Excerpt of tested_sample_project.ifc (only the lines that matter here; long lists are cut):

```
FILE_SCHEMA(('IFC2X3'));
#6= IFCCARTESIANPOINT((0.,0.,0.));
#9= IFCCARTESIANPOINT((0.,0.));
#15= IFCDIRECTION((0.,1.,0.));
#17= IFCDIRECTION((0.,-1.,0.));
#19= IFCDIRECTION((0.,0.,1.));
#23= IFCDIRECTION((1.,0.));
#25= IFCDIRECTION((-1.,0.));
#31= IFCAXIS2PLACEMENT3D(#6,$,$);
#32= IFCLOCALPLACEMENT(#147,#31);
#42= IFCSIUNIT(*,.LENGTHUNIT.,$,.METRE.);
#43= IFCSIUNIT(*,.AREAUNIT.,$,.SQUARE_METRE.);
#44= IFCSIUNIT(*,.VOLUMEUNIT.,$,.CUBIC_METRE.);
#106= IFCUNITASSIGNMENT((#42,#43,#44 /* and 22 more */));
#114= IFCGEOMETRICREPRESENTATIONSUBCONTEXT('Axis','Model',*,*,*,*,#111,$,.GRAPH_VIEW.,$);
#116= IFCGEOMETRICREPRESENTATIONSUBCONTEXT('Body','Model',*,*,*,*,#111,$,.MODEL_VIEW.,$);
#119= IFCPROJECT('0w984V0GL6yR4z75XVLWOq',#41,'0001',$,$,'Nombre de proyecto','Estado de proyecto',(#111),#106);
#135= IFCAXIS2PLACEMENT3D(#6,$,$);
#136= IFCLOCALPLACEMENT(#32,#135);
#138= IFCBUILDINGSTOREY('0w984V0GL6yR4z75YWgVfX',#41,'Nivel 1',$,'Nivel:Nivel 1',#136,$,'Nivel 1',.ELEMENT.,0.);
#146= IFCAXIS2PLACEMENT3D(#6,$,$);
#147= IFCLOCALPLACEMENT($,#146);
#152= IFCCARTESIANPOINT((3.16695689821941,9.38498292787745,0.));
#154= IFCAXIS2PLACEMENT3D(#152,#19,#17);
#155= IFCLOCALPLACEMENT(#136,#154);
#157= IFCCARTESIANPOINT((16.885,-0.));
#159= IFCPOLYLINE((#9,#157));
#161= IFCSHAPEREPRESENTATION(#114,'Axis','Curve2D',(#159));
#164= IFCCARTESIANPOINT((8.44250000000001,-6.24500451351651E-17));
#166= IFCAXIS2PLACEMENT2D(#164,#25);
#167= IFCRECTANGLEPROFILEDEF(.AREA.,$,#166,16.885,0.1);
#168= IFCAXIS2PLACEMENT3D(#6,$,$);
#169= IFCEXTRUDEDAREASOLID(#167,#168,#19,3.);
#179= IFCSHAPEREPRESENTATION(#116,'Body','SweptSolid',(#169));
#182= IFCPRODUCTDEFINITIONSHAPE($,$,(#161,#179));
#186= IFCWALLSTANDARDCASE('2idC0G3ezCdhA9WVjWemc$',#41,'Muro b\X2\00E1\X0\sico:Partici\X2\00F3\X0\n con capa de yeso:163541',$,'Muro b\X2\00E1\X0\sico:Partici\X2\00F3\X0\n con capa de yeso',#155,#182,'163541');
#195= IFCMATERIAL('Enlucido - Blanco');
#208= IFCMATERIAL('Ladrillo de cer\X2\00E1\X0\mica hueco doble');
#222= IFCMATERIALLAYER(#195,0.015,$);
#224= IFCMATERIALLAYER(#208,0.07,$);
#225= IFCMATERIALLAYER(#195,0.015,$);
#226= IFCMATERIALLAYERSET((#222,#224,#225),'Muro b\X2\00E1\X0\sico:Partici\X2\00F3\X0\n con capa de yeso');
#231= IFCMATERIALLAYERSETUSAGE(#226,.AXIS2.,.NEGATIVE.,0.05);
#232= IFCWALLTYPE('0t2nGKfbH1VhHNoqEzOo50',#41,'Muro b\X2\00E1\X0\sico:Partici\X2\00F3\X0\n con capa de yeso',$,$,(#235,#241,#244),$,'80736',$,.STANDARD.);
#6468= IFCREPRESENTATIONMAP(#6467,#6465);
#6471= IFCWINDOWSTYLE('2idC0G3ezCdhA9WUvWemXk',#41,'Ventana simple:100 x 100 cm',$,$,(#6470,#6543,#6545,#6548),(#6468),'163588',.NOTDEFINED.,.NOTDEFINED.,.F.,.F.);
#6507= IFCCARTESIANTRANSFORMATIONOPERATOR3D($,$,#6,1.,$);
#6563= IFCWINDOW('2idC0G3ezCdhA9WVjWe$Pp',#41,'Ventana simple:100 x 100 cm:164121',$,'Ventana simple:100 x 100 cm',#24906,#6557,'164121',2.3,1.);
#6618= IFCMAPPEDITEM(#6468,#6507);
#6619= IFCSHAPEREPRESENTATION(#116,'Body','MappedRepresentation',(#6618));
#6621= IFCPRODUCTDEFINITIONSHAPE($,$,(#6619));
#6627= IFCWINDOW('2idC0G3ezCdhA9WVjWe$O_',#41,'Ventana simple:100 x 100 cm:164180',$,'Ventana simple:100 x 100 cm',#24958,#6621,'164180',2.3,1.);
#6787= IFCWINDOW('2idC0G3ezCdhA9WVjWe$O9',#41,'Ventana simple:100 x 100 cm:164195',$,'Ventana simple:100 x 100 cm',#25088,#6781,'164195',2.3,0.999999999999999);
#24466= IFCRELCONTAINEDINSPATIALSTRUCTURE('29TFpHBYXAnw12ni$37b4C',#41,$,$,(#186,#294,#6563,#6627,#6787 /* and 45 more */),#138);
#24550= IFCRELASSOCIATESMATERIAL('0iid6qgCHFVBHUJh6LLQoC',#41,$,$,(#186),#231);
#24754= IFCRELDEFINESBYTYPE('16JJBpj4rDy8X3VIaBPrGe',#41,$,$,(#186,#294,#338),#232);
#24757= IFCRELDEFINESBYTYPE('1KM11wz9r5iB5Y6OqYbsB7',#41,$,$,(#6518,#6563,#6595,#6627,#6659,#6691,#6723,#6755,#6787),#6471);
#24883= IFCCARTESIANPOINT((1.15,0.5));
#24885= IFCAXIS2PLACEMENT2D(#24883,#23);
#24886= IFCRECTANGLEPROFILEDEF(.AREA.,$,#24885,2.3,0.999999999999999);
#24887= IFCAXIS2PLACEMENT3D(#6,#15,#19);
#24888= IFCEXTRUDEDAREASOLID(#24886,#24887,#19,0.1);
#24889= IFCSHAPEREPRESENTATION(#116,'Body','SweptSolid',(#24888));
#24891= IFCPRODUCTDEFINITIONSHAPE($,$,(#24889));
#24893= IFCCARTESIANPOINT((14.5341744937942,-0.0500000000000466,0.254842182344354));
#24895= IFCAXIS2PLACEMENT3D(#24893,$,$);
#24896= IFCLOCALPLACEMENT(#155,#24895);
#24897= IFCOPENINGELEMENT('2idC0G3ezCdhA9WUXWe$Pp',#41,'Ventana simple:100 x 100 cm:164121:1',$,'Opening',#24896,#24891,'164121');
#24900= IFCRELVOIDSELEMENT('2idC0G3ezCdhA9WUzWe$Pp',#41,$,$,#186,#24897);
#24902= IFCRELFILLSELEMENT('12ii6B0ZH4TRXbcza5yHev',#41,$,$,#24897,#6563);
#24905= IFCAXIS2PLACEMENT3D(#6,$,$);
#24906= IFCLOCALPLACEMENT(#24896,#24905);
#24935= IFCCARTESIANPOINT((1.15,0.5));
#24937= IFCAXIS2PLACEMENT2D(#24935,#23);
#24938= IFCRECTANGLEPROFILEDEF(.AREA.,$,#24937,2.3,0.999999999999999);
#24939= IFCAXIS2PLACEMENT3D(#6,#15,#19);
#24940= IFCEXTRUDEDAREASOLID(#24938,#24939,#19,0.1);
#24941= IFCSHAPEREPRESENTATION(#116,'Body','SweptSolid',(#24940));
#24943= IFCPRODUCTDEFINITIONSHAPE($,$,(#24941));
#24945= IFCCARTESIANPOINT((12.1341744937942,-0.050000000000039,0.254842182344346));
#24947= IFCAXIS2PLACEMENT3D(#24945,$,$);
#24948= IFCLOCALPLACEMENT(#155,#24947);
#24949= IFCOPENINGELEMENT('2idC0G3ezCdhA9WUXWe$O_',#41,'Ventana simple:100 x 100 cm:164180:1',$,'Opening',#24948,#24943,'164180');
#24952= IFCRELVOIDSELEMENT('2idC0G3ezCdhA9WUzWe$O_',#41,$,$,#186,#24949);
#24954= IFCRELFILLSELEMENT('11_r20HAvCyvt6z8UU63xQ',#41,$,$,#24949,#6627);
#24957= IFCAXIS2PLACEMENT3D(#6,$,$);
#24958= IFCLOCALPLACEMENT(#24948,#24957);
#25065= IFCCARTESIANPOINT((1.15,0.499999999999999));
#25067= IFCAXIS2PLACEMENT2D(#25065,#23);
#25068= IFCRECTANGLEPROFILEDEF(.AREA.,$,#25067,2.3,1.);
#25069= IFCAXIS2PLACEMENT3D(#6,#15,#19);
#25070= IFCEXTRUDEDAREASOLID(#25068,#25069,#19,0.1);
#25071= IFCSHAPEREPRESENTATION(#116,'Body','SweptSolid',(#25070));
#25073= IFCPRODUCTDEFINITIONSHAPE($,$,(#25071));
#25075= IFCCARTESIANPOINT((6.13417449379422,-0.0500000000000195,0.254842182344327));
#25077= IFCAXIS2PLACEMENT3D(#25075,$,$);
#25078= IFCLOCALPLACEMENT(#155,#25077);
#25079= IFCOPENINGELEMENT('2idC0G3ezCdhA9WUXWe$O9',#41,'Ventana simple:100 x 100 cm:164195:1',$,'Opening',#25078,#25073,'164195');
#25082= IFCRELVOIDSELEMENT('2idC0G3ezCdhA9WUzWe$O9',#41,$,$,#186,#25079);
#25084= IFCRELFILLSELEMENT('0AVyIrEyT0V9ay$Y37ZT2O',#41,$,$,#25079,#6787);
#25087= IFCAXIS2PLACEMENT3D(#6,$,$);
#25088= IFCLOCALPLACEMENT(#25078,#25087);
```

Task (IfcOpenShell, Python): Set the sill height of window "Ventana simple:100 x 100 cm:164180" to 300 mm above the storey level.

```python
import numpy as np
import ifcopenshell
import ifcopenshell.api.geometry
import ifcopenshell.geom
import ifcopenshell.util.element
import ifcopenshell.util.placement
import ifcopenshell.util.shape
import ifcopenshell.util.unit

model = ifcopenshell.open("tested_sample_project.ifc")
unit_scale = ifcopenshell.util.unit.calculate_unit_scale(model)

window = model.by_guid("2idC0G3ezCdhA9WVjWe$O_")
opening = window.FillsVoids[0].RelatingOpeningElement
storey = ifcopenshell.util.element.get_container(window, ifc_class="IfcBuildingStorey")
level = ifcopenshell.util.placement.get_local_placement(storey.ObjectPlacement)[2, 3]

# The opening's origin need not be at the sill, so measure its lowest point.
shape = ifcopenshell.geom.create_shape(ifcopenshell.geom.settings(), opening)
bottom = ifcopenshell.util.shape.get_shape_bottom_elevation(shape, shape.geometry) / unit_scale
dz = level + 0.3 - bottom

shift = np.array([0.0, 0.0, dz])
# The window is placed relative to its opening, so it follows when the opening moves.
matrix = ifcopenshell.util.placement.get_local_placement(opening.ObjectPlacement)
matrix[:3, 3] += shift
ifcopenshell.api.geometry.edit_object_placement(
    model, product=opening, matrix=matrix, is_si=False, should_transform_children=True
)

print(f"moved by {dz * unit_scale:+.3f} m")

model.write("tested_sample_project_rev.ifc")
```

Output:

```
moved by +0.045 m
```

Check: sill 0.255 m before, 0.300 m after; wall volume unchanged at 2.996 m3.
